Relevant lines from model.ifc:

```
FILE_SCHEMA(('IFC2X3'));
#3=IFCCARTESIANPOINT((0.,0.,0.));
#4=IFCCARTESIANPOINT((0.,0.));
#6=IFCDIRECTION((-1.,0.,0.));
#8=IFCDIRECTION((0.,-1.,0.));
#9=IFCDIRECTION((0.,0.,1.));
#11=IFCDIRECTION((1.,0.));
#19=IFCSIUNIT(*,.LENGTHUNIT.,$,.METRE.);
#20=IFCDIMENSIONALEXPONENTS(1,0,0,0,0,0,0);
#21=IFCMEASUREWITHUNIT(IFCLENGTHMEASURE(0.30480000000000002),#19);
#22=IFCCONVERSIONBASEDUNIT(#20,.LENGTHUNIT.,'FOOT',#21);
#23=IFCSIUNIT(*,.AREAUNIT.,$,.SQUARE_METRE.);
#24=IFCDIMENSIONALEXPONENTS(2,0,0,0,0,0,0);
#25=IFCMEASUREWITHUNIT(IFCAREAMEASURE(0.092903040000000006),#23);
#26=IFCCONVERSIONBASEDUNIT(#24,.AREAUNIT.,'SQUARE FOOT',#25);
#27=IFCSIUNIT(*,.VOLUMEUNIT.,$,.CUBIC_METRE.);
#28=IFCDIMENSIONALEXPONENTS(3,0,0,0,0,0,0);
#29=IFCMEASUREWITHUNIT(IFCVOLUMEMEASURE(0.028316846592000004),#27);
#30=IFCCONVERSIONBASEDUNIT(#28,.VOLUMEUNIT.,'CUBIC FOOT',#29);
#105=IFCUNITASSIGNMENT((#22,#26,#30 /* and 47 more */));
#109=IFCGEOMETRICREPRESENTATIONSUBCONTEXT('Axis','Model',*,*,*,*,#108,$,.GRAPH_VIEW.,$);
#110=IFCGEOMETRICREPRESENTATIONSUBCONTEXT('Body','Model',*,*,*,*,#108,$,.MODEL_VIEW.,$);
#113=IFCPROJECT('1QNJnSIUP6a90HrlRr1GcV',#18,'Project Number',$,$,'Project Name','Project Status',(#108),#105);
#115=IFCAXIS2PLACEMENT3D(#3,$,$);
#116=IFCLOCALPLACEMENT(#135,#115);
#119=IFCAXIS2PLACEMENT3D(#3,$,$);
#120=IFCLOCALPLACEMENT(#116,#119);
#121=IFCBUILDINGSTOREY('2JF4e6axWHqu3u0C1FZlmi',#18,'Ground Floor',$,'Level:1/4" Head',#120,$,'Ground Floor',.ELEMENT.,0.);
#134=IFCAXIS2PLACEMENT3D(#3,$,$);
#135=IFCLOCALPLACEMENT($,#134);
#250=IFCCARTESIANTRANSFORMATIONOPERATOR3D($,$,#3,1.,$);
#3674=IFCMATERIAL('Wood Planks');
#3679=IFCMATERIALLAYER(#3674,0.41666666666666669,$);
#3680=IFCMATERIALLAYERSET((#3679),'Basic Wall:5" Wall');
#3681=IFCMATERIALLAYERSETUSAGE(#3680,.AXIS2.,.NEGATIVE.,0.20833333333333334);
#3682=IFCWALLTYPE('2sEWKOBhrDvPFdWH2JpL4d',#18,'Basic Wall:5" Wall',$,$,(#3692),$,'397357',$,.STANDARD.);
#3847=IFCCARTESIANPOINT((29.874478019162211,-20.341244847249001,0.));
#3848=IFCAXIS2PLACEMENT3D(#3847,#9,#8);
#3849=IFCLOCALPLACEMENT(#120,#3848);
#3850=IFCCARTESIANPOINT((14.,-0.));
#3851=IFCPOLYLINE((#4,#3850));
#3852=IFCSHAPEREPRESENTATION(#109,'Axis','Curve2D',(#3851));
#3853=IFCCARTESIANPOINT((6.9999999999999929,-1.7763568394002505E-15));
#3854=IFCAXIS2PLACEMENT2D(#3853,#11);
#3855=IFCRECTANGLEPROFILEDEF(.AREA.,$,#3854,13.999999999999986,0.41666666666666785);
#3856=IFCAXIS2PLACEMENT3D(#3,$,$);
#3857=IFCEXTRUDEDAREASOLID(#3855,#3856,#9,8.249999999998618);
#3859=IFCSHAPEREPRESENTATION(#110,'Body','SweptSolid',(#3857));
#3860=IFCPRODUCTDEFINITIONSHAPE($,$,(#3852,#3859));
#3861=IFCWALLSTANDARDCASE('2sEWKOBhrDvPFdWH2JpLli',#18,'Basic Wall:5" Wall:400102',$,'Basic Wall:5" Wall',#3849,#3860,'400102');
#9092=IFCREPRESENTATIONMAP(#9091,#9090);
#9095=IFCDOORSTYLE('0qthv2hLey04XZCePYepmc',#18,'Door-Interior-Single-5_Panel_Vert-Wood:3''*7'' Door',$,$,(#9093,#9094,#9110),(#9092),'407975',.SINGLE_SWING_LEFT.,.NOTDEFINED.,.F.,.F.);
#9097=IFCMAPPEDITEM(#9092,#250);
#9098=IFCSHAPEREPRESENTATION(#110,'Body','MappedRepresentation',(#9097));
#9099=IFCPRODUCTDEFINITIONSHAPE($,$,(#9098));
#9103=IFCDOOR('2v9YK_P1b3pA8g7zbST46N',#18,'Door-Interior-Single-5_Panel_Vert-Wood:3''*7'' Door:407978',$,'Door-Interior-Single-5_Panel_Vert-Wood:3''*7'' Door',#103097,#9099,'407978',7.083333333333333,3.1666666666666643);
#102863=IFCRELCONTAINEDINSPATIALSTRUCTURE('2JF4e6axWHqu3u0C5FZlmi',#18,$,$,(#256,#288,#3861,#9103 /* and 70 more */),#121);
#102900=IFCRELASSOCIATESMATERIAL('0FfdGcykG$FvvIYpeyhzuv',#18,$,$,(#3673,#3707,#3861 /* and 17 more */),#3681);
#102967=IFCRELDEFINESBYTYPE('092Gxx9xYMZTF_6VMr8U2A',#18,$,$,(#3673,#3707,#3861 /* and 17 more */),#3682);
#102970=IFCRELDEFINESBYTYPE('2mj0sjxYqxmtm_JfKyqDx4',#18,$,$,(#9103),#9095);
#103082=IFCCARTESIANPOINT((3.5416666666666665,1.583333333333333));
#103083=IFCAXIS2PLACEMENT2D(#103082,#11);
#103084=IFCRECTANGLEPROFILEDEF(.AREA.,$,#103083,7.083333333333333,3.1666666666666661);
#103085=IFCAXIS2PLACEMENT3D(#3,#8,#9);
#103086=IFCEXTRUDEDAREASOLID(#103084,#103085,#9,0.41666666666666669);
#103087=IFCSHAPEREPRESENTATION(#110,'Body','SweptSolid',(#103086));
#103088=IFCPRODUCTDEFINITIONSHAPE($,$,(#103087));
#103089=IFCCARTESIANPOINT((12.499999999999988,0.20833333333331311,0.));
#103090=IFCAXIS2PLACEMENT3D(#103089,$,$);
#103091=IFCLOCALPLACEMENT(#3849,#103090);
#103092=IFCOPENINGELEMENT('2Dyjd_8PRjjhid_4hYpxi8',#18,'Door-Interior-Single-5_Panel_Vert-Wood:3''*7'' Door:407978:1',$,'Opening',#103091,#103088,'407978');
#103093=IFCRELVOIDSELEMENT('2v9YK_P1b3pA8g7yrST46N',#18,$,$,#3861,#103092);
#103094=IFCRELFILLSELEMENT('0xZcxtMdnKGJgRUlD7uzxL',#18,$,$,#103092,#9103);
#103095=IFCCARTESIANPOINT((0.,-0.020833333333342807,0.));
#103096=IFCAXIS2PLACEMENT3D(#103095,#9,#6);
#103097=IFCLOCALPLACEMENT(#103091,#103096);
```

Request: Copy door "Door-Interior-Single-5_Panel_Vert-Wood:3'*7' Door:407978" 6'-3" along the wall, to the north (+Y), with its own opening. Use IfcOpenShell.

```python
import ifcopenshell
import ifcopenshell.api.feature
import ifcopenshell.api.geometry
import ifcopenshell.api.root
import ifcopenshell.geom
import ifcopenshell.util.element
import ifcopenshell.util.placement
import ifcopenshell.util.shape
import ifcopenshell.util.unit

model = ifcopenshell.open("model.ifc")
unit_scale = ifcopenshell.util.unit.calculate_unit_scale(model)
settings = ifcopenshell.geom.settings()


def volume(element):
    """Net volume in cubic metres, openings subtracted."""
    shape = ifcopenshell.geom.create_shape(settings, element)
    return ifcopenshell.util.shape.get_volume(shape.geometry)


def reuse_history(source, copy):
    """copy_class also copies each property set's owner history, people and application; keep the originals."""
    for rel in copy.IsDefinedBy:
        if rel.is_a("IfcRelDefinesByProperties") and (history := rel.RelatingPropertyDefinition.OwnerHistory):
            rel.RelatingPropertyDefinition.OwnerHistory = source.OwnerHistory
            ifcopenshell.util.element.remove_deep2(model, history)


door = model.by_guid("2v9YK_P1b3pA8g7zbST46N")
opening = door.FillsVoids[0].RelatingOpeningElement
wall = opening.VoidsElements[0].RelatingBuildingElement
before = volume(wall)
shift = ifcopenshell.util.placement.get_local_placement(wall.ObjectPlacement)[:3, 0] * -75 * 0.0254 / unit_scale

# copy_class copies the void relationship, type, container and properties, but no geometry.
new_opening = ifcopenshell.api.root.copy_class(model, product=opening)
new_opening.Representation = ifcopenshell.util.element.copy_deep(
    model, opening.Representation, exclude=["IfcGeometricRepresentationContext", "IfcRepresentationMap"]
)
new_opening.Name = "Door-Interior-Single-5_Panel_Vert-Wood:3'*7' Door"
new_opening.Tag = None
new_door = ifcopenshell.api.root.copy_class(model, product=door)
new_door.Representation = ifcopenshell.util.element.copy_deep(
    model, door.Representation, exclude=["IfcGeometricRepresentationContext", "IfcRepresentationMap"]
)
new_door.Name = "Door-Interior-Single-5_Panel_Vert-Wood:3'*7' Door"
new_door.Tag = None
reuse_history(door, new_door)
fills = ifcopenshell.api.feature.add_filling(model, opening=new_opening, element=new_door)
fills.OwnerHistory = new_door.OwnerHistory  # required in IFC2X3

for old, new in ((opening, new_opening), (door, new_door)):
    matrix = ifcopenshell.util.placement.get_local_placement(old.ObjectPlacement)
    matrix[:3, 3] += shift
    ifcopenshell.api.geometry.edit_object_placement(model, product=new, matrix=matrix, is_si=False)

after = volume(wall)

print(f"wall volume {before:.3f} -> {after:.3f} m3")

model.write("model_updated.ifc")
```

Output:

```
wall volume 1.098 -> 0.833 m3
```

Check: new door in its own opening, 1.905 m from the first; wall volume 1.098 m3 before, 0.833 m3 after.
